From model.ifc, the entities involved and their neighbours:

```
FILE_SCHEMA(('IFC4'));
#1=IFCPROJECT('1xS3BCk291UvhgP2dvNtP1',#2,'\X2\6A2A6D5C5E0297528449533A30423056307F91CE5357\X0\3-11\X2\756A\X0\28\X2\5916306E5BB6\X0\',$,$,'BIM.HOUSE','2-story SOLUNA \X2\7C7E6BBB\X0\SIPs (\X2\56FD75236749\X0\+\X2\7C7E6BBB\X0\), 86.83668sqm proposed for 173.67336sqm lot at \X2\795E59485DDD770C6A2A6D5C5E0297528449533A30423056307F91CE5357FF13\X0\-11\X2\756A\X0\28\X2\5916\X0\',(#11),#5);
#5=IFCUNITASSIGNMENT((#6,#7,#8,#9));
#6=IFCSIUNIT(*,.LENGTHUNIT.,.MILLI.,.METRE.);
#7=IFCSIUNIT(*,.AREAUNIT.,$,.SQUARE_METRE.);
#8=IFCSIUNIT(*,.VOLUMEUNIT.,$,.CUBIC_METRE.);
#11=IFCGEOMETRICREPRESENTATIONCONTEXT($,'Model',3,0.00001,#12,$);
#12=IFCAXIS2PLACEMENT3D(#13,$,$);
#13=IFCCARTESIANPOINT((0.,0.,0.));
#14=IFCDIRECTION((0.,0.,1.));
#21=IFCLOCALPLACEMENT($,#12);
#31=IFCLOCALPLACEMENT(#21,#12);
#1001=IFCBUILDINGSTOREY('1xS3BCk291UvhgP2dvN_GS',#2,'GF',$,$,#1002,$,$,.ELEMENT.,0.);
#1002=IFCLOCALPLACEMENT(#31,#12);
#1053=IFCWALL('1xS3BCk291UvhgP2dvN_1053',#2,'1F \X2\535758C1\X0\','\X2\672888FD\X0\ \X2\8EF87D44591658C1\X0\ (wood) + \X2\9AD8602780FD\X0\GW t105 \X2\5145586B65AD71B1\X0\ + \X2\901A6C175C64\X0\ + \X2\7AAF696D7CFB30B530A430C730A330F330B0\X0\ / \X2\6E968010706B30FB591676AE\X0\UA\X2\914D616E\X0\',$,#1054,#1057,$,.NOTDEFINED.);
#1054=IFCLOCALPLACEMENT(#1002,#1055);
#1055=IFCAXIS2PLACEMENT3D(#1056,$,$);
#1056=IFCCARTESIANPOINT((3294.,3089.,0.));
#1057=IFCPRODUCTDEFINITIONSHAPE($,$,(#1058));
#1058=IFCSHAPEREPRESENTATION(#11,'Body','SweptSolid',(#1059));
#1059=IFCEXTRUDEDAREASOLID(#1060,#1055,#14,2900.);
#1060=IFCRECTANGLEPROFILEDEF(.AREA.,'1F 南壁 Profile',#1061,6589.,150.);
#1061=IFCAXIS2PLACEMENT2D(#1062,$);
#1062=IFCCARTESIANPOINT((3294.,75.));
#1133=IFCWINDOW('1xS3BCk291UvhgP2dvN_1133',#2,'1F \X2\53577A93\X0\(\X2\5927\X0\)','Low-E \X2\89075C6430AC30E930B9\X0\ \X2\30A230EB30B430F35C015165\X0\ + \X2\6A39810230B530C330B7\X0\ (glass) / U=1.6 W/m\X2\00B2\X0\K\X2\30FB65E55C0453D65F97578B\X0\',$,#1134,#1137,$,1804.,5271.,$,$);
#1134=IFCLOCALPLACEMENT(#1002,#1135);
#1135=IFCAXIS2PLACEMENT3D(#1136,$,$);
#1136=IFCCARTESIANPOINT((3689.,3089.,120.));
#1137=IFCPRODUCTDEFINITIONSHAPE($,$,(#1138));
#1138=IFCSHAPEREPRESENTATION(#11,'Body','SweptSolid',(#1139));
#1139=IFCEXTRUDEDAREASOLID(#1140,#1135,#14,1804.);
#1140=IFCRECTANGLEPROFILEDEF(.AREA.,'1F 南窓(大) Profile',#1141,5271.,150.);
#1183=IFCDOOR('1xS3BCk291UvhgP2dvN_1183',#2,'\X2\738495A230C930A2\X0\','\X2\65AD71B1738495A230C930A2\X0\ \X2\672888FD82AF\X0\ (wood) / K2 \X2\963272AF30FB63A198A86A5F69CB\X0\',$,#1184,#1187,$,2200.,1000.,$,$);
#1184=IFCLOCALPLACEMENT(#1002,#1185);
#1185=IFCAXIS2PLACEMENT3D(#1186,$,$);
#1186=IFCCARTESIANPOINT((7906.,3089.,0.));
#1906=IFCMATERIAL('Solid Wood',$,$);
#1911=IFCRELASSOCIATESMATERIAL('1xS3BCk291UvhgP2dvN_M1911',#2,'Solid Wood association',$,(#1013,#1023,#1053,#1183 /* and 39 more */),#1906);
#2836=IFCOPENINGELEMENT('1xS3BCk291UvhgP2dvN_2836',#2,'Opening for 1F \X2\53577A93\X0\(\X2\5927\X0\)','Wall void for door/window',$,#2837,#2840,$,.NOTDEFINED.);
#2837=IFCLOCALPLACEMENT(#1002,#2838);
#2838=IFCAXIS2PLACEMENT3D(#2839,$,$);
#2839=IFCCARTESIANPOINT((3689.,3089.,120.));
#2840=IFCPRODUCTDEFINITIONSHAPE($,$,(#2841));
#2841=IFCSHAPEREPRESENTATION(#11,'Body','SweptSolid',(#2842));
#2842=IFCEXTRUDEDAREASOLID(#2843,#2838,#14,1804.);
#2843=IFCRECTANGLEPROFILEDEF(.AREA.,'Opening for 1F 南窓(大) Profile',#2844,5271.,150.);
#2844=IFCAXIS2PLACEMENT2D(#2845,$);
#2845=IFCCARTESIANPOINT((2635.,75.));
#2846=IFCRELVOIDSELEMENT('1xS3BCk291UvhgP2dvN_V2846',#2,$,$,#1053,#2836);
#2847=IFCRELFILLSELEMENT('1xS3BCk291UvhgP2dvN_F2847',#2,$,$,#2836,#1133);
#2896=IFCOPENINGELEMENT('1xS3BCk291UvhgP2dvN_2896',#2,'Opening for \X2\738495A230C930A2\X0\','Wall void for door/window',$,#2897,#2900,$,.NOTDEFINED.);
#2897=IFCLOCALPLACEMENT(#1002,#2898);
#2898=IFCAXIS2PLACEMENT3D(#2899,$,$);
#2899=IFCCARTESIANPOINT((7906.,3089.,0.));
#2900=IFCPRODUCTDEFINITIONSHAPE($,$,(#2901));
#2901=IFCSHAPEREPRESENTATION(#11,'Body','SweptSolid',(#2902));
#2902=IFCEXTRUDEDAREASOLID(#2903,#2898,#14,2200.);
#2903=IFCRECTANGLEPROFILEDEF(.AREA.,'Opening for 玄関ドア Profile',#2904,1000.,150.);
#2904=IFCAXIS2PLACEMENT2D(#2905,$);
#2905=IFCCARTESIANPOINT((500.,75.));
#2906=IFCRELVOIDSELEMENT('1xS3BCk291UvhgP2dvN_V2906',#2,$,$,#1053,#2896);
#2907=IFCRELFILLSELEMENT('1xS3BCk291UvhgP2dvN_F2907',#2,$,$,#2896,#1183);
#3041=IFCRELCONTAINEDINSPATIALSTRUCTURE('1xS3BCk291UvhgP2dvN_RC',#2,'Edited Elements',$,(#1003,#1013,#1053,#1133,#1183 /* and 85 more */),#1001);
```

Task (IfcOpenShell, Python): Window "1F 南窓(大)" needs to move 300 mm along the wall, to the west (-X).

```python
import ifcopenshell
import ifcopenshell.api.geometry
import ifcopenshell.util.placement
import ifcopenshell.util.unit

model = ifcopenshell.open("model.ifc")
unit_scale = ifcopenshell.util.unit.calculate_unit_scale(model)

window = model.by_id(1133)
opening = window.FillsVoids[0].RelatingOpeningElement
wall = opening.VoidsElements[0].RelatingBuildingElement

wall_matrix = ifcopenshell.util.placement.get_local_placement(wall.ObjectPlacement)
shift = wall_matrix[:3, 0] * -0.3 / unit_scale
before = ifcopenshell.util.placement.get_local_placement(window.ObjectPlacement)[:3, 3].copy()

# The window is not placed relative to its opening, so move both.
for product in (opening, window):
    matrix = ifcopenshell.util.placement.get_local_placement(product.ObjectPlacement)
    matrix[:3, 3] += shift
    ifcopenshell.api.geometry.edit_object_placement(model, product=product, matrix=matrix, is_si=False)

after = ifcopenshell.util.placement.get_local_placement(window.ObjectPlacement)[:3, 3]
print("window moved by", (after - before).round(3) + 0.0)

model.write("model-out.ifc")
```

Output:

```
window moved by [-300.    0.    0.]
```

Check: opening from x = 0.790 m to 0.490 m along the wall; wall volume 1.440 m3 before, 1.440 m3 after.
